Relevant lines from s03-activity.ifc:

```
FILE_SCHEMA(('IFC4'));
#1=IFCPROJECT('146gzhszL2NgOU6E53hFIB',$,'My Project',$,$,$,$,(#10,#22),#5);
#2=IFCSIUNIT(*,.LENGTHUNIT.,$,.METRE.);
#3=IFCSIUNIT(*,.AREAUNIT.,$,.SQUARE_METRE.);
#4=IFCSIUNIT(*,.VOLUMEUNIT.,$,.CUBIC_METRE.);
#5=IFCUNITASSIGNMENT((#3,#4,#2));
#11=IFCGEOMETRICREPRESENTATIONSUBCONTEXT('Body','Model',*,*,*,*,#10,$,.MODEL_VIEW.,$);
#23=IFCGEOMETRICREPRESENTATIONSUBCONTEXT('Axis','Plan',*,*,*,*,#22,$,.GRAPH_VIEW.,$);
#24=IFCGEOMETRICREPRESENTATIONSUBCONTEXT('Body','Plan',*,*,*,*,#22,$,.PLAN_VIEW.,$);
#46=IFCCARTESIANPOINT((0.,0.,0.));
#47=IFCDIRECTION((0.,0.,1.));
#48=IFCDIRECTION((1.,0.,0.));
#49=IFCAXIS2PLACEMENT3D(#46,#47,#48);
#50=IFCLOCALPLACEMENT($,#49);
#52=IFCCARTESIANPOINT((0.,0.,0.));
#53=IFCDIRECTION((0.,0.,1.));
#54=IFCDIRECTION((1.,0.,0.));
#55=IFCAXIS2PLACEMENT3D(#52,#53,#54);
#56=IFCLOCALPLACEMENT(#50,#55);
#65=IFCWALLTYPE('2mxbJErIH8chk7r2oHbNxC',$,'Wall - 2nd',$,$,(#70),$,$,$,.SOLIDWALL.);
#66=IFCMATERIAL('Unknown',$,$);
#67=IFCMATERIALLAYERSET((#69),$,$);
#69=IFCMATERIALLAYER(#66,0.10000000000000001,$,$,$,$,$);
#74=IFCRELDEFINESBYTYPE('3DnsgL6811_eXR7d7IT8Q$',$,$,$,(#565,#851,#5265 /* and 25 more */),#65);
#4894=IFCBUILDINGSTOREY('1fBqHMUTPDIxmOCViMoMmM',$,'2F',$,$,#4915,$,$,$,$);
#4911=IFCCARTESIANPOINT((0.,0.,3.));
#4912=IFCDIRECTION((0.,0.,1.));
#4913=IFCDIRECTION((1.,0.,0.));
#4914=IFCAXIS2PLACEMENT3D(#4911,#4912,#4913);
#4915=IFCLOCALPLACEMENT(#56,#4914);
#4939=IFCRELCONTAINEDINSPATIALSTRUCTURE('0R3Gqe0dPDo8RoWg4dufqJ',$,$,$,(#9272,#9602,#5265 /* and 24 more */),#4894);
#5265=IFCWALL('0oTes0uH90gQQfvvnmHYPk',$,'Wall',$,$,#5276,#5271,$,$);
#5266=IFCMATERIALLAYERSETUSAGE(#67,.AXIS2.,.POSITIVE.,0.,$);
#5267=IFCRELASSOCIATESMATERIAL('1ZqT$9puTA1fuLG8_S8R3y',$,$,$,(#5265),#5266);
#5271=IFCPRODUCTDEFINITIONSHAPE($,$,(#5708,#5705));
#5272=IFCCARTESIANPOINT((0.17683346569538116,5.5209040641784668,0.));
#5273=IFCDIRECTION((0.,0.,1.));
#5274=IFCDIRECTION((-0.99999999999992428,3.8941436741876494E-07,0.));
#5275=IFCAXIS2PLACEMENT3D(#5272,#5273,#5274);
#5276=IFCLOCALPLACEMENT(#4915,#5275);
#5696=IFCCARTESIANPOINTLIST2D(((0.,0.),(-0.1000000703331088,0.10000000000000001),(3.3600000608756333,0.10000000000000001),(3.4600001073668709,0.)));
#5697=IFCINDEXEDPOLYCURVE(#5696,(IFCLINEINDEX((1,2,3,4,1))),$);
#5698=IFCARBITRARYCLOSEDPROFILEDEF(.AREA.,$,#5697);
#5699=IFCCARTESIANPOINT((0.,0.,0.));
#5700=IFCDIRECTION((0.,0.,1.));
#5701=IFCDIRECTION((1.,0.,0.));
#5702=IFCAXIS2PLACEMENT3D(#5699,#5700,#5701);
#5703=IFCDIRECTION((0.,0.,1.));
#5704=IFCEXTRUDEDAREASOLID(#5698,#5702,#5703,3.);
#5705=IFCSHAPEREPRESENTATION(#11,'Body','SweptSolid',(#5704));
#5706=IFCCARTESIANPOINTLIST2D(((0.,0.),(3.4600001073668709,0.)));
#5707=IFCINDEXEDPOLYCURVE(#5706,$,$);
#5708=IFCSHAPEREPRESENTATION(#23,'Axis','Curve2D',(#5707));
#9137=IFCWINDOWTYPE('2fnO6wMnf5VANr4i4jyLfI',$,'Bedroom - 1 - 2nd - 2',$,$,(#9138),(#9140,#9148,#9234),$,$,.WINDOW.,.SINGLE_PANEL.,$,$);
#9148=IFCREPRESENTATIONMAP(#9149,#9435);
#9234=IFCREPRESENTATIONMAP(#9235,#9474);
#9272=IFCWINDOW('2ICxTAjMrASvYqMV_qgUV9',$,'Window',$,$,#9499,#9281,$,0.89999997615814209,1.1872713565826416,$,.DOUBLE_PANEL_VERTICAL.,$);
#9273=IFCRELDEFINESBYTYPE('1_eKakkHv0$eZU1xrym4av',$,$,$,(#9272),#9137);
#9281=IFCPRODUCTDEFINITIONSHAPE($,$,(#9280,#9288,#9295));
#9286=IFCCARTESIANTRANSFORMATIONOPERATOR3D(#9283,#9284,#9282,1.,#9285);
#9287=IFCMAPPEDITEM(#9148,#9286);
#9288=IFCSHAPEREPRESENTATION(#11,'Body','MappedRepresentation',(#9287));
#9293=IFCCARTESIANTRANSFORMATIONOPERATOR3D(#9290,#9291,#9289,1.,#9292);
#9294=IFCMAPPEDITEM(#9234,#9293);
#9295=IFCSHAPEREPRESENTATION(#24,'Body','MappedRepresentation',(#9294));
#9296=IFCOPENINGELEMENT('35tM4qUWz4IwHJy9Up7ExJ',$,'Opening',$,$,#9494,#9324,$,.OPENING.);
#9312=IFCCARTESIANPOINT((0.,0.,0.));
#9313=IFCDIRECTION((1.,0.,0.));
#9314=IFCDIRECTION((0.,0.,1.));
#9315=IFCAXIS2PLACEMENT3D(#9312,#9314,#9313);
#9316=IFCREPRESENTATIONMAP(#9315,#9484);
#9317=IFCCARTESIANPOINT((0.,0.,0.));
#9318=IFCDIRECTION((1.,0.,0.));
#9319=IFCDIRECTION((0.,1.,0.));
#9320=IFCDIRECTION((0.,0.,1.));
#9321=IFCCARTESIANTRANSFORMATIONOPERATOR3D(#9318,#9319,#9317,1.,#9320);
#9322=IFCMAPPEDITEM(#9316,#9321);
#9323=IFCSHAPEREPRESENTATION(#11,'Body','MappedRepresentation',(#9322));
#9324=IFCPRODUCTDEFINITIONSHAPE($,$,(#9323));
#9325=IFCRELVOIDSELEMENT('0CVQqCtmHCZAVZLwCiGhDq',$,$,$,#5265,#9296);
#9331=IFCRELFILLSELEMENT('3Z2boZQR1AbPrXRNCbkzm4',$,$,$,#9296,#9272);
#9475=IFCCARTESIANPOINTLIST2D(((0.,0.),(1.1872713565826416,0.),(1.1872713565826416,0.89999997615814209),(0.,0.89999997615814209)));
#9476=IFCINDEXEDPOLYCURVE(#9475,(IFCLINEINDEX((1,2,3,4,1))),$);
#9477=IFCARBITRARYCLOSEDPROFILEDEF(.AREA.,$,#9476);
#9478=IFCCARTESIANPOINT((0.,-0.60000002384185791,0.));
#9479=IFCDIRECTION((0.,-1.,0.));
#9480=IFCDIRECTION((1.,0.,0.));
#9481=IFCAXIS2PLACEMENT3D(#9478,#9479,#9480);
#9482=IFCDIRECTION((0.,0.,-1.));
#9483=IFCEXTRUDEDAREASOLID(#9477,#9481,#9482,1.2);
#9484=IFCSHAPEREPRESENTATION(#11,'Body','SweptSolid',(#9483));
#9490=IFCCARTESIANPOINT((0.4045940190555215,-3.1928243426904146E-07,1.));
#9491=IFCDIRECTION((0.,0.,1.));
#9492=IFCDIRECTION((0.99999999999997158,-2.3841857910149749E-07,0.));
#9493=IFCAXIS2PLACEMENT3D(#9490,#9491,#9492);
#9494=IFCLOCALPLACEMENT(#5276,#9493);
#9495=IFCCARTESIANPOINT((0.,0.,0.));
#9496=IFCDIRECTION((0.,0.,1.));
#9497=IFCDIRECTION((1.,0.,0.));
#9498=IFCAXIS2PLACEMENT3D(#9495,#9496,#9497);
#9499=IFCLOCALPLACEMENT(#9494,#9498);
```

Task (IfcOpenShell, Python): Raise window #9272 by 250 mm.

```python
import numpy as np
import ifcopenshell
import ifcopenshell.api.geometry
import ifcopenshell.util.placement
import ifcopenshell.util.unit

model = ifcopenshell.open("s03-activity.ifc")
unit_scale = ifcopenshell.util.unit.calculate_unit_scale(model)

window = model.by_id(9272)
opening = window.FillsVoids[0].RelatingOpeningElement
dz = 0.25

shift = np.array([0.0, 0.0, dz])
# The window is placed relative to its opening, so it follows when the opening moves.
matrix = ifcopenshell.util.placement.get_local_placement(opening.ObjectPlacement)
matrix[:3, 3] += shift
ifcopenshell.api.geometry.edit_object_placement(
    model, product=opening, matrix=matrix, is_si=False, should_transform_children=True
)

print(f"moved by {dz * unit_scale:+.3f} m")

model.write("s03-activity_updated.ifc")
```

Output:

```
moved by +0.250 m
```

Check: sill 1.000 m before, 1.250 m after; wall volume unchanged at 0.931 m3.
